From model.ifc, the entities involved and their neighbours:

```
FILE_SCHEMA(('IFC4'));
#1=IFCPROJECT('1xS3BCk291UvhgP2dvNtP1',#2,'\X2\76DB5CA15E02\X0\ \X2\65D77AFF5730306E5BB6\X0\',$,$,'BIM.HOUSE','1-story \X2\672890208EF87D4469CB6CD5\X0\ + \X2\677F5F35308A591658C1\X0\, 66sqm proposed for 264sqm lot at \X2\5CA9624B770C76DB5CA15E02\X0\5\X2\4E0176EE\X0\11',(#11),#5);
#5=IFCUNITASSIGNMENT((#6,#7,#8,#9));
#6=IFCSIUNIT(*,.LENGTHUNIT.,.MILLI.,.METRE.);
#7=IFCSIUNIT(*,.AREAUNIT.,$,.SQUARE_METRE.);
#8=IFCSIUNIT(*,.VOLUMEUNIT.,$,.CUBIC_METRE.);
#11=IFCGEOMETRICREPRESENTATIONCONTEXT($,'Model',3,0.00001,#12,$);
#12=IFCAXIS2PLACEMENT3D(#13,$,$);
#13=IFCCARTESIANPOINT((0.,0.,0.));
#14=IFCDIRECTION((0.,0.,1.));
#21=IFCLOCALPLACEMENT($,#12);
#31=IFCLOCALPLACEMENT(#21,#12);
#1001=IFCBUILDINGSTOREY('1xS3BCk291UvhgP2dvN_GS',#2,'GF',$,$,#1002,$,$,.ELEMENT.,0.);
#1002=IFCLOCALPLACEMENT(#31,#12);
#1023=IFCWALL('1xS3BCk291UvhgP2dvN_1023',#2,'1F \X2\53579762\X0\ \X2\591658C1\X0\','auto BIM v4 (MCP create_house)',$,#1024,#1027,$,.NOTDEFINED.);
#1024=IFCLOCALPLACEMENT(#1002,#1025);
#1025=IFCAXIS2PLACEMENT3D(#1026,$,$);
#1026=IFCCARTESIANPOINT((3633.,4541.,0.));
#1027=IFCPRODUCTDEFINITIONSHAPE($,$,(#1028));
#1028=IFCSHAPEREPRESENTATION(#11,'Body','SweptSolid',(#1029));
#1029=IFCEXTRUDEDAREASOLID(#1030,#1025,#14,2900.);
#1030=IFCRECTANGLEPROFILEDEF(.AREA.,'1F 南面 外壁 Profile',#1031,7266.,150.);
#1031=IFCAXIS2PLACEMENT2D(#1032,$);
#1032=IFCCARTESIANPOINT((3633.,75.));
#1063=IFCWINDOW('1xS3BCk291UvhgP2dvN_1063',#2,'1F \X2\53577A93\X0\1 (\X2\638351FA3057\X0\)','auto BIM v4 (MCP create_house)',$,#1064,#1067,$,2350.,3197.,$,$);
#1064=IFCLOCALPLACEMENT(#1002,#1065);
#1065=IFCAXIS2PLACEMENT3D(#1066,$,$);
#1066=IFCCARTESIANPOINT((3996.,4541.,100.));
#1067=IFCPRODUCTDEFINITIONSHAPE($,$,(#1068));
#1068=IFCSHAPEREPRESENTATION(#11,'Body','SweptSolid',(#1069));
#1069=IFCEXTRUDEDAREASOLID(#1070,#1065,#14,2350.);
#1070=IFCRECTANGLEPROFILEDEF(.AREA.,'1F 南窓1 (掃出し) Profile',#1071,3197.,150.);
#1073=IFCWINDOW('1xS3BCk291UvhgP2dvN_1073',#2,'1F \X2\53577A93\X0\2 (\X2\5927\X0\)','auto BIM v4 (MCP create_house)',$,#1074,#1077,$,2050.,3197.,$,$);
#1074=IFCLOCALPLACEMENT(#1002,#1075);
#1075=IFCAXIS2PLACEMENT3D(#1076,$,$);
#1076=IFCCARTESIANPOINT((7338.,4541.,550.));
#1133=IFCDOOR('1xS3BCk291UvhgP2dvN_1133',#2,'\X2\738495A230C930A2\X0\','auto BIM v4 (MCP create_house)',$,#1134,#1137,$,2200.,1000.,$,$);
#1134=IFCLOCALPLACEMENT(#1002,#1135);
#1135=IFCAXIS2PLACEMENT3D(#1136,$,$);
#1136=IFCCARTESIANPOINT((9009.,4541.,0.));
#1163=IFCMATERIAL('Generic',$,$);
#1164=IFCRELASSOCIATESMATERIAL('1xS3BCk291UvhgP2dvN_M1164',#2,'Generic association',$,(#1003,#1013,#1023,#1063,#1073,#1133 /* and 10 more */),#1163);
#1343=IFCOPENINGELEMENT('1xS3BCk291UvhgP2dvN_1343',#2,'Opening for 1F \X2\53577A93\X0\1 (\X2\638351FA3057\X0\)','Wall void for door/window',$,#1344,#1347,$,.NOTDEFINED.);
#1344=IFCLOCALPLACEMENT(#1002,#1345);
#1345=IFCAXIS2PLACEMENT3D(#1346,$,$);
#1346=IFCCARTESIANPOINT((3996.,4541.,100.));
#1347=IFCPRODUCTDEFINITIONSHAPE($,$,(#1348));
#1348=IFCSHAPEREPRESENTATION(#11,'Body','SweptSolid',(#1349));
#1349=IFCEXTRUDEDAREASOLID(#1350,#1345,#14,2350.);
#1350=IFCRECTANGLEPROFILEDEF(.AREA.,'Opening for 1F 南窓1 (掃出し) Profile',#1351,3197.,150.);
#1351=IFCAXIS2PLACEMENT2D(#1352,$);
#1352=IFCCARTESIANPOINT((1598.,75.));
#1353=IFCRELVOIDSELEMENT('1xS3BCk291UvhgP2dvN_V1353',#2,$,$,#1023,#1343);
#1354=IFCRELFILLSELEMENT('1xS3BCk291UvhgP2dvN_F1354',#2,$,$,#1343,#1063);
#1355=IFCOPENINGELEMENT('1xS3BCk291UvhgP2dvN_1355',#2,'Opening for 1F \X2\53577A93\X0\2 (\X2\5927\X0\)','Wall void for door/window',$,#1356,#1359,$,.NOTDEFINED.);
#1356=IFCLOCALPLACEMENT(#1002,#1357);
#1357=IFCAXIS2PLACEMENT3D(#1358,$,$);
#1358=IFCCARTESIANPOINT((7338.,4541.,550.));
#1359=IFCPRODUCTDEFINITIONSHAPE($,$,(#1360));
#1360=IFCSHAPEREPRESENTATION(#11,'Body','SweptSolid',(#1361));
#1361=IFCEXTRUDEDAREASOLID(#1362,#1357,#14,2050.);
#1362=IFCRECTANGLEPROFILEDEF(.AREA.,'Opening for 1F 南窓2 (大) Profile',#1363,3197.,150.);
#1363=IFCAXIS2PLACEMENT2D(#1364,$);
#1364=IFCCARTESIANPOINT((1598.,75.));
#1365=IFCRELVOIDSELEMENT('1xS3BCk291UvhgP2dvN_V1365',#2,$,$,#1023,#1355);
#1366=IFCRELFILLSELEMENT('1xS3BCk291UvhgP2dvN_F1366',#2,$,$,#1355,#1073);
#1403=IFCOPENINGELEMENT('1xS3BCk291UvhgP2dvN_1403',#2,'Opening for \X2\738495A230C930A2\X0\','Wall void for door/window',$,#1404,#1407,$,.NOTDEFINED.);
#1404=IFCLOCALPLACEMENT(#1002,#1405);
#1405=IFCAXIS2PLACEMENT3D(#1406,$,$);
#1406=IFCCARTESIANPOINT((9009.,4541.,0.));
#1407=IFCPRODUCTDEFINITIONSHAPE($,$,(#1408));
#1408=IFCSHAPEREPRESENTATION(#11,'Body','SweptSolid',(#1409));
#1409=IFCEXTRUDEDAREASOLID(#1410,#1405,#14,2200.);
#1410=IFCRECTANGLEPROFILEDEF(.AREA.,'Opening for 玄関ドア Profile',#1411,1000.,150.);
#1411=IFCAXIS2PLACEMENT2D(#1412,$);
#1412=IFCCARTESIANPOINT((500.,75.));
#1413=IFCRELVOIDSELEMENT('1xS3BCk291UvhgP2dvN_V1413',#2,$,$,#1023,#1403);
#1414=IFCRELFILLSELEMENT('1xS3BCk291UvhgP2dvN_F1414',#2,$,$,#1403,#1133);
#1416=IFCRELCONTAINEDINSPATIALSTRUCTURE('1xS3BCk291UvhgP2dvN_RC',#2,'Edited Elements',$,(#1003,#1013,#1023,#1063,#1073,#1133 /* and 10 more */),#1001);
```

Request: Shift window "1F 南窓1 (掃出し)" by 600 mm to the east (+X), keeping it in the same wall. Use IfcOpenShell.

```python
import ifcopenshell
import ifcopenshell.api.geometry
import ifcopenshell.util.placement

model = ifcopenshell.open("model.ifc")

window = model.by_guid("1xS3BCk291UvhgP2dvN_1063")
opening = window.FillsVoids[0].RelatingOpeningElement
wall = opening.VoidsElements[0].RelatingBuildingElement

wall_matrix = ifcopenshell.util.placement.get_local_placement(wall.ObjectPlacement)
shift = wall_matrix[:3, 0] * 600.0
before = ifcopenshell.util.placement.get_local_placement(window.ObjectPlacement)[:3, 3].copy()

# The window is not placed relative to its opening, so move both.
for product in (opening, window):
    matrix = ifcopenshell.util.placement.get_local_placement(product.ObjectPlacement)
    matrix[:3, 3] += shift
    ifcopenshell.api.geometry.edit_object_placement(model, product=product, matrix=matrix, is_si=False)

after = ifcopenshell.util.placement.get_local_placement(window.ObjectPlacement)[:3, 3]
print("window moved by", (after - before).round(3) + 0.0)

model.write("model_rev.ifc")
```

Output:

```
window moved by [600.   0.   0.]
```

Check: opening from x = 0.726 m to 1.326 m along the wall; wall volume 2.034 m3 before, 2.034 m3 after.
